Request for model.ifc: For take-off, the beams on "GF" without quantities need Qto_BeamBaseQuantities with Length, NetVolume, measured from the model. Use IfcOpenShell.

First a look at what the model holds.

```python
import ifcopenshell
import ifcopenshell.util.element
import ifcopenshell.util.unit

model = ifcopenshell.open("model.ifc")
print(model.schema)
for unit_type in ("LENGTHUNIT", "AREAUNIT", "VOLUMEUNIT"):
    print(unit_type, ifcopenshell.util.unit.calculate_unit_scale(model, unit_type))
storey = next(s for s in model.by_type("IfcBuildingStorey") if s.Name == "GF")
beams = [e for e in ifcopenshell.util.element.get_decomposition(storey) if e.is_a("IfcBeam")]
for e in sorted(beams, key=lambda e: e.id()):
    print(e.id(), e.is_a(), e.Name, list(ifcopenshell.util.element.get_psets(e, qtos_only=True)), sep=" | ")
```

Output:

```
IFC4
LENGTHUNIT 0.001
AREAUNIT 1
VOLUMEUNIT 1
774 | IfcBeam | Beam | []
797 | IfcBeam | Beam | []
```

```python
import ifcopenshell
import ifcopenshell.api.pset
import ifcopenshell.geom
import ifcopenshell.util.element
import ifcopenshell.util.shape
import ifcopenshell.util.unit

model = ifcopenshell.open("model.ifc")
unit_scale = ifcopenshell.util.unit.calculate_unit_scale(model)
volume_scale = ifcopenshell.util.unit.calculate_unit_scale(model, "VOLUMEUNIT")
settings = ifcopenshell.geom.settings()

storey = next(s for s in model.by_type("IfcBuildingStorey") if s.Name == "GF")
beams = [e for e in ifcopenshell.util.element.get_decomposition(storey) if e.is_a("IfcBeam")]

for e in sorted(beams, key=lambda e: e.id()):
    if ifcopenshell.util.element.get_psets(e, qtos_only=True, should_inherit=False):
        continue
    # Geometry comes back in metres, in the element's own axes.
    shape = ifcopenshell.geom.create_shape(settings, e)
    values = {
        "Length": ifcopenshell.util.shape.get_max_xyz(shape.geometry) / unit_scale,
        "NetVolume": ifcopenshell.util.shape.get_volume(shape.geometry) / volume_scale,
    }
    qto = ifcopenshell.api.pset.add_qto(model, product=e, name="Qto_BeamBaseQuantities")
    ifcopenshell.api.pset.edit_qto(model, qto=qto, properties=values)
    print(e.id(), {k: round(v, 3) for k, v in values.items()})

model.write("model-out.ifc")
```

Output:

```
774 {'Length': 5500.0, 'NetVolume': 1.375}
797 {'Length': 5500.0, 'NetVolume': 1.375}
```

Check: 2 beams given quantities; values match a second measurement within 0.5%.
